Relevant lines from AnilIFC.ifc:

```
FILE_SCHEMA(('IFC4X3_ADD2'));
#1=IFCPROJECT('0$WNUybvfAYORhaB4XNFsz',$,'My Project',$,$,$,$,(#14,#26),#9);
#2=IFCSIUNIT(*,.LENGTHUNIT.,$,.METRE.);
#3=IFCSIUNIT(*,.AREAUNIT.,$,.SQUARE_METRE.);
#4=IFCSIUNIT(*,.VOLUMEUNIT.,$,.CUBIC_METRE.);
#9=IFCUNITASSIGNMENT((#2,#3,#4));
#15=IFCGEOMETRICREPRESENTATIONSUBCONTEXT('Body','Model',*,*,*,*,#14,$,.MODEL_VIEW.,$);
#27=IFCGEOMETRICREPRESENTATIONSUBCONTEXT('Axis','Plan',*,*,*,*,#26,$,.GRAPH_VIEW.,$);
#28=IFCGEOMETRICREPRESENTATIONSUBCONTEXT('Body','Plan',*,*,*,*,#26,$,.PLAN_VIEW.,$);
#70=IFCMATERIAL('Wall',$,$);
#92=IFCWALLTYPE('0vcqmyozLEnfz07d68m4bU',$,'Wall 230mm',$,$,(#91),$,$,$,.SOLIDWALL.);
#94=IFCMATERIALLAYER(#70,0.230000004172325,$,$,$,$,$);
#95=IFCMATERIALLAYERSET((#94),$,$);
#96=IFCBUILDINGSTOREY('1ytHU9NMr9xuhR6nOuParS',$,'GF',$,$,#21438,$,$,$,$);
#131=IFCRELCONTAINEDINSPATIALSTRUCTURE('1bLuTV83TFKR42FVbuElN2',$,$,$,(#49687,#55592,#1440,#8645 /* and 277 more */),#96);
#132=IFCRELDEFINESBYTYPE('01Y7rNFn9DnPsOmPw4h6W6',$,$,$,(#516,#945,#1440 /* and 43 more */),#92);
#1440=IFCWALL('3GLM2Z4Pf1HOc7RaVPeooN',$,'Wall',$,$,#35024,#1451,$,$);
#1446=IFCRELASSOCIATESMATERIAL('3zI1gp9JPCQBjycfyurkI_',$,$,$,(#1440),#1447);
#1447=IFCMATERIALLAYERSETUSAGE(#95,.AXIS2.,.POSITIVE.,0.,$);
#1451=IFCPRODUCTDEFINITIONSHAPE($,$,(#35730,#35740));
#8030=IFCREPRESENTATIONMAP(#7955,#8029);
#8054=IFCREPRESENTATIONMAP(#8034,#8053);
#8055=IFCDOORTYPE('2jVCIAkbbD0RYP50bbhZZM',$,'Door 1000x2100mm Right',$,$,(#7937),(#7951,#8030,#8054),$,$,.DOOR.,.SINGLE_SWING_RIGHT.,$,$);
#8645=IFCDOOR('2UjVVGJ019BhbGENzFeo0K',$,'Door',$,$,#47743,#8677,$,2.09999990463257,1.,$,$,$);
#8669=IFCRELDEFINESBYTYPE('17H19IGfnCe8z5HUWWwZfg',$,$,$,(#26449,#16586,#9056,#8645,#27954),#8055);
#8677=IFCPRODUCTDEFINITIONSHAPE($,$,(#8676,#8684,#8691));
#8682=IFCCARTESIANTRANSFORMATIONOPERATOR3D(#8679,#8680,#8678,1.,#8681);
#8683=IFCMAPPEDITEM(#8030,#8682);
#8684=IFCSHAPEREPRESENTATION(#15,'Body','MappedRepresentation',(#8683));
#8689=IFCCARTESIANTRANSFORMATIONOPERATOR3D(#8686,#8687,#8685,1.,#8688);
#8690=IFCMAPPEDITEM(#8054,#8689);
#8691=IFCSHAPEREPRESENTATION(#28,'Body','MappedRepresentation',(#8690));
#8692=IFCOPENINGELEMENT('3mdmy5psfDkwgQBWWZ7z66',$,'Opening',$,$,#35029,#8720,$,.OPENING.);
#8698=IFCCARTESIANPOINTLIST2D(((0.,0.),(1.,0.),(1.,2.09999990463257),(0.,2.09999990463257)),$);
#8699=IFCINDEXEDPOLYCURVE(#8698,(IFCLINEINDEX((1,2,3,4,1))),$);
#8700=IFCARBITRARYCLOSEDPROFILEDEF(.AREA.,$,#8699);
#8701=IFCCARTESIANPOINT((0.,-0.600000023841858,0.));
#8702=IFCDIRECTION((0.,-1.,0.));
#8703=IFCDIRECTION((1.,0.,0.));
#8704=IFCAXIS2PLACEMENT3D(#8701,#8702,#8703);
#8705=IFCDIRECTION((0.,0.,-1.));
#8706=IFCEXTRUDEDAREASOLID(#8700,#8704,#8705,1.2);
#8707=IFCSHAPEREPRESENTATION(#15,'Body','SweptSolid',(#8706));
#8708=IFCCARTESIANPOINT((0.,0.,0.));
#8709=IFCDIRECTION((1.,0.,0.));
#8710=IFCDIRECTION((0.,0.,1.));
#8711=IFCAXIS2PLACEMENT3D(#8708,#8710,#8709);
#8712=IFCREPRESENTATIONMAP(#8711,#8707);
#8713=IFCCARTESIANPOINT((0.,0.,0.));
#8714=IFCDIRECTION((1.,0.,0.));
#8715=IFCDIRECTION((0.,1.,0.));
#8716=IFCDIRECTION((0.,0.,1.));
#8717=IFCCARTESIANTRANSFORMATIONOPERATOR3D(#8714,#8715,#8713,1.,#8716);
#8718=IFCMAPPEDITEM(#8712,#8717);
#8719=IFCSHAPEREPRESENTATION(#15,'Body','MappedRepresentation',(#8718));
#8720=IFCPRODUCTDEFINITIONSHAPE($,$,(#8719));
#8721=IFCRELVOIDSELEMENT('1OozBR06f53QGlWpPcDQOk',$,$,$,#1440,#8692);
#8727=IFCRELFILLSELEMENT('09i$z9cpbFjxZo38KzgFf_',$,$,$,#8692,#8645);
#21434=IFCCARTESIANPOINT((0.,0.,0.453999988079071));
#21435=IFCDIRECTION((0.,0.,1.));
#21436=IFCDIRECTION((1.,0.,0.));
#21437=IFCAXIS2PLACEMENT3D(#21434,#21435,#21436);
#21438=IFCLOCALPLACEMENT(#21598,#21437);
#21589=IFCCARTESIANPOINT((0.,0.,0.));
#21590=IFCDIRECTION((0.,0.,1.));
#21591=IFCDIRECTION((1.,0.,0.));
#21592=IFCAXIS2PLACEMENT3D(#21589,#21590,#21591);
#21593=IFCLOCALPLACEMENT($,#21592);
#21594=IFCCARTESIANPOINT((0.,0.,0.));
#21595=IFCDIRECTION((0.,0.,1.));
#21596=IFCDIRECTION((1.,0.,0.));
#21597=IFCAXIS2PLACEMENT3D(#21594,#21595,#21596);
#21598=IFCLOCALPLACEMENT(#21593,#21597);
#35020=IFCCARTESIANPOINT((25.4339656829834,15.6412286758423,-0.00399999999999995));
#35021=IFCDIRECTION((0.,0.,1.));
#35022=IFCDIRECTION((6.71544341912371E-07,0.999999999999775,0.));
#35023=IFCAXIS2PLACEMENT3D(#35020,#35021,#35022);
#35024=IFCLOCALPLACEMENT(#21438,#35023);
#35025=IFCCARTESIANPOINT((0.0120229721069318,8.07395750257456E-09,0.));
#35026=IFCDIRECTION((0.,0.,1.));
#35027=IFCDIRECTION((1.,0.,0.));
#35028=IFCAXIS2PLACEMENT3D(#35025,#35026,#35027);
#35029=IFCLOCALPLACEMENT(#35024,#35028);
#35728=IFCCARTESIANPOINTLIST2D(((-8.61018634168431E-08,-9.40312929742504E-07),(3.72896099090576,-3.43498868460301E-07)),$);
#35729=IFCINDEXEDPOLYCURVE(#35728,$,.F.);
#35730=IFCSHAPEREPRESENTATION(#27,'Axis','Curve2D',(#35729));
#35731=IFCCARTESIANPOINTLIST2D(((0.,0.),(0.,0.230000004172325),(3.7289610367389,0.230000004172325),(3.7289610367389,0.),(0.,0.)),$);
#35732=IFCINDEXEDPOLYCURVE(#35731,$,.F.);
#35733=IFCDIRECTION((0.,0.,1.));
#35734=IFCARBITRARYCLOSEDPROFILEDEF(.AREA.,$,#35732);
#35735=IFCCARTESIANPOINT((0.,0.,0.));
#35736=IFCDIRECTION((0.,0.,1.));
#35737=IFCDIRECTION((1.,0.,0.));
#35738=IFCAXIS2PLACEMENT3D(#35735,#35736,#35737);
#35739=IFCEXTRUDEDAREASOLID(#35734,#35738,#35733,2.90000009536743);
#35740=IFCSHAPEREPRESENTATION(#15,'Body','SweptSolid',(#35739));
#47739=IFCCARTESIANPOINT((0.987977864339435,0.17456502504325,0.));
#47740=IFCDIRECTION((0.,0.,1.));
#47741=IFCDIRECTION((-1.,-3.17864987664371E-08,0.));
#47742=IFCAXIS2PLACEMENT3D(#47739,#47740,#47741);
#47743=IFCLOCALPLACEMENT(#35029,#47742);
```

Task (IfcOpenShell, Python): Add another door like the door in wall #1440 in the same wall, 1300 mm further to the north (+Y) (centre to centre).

```python
import ifcopenshell
import ifcopenshell.api.feature
import ifcopenshell.api.geometry
import ifcopenshell.api.root
import ifcopenshell.geom
import ifcopenshell.util.element
import ifcopenshell.util.placement
import ifcopenshell.util.shape
import ifcopenshell.util.unit

model = ifcopenshell.open("AnilIFC.ifc")
unit_scale = ifcopenshell.util.unit.calculate_unit_scale(model)
settings = ifcopenshell.geom.settings()


def volume(element):
    """Net volume in cubic metres, openings subtracted."""
    shape = ifcopenshell.geom.create_shape(settings, element)
    return ifcopenshell.util.shape.get_volume(shape.geometry)


door = model.by_guid("2UjVVGJ019BhbGENzFeo0K")
opening = door.FillsVoids[0].RelatingOpeningElement
wall = opening.VoidsElements[0].RelatingBuildingElement
before = volume(wall)
shift = ifcopenshell.util.placement.get_local_placement(wall.ObjectPlacement)[:3, 0] * 1.3 / unit_scale

# copy_class copies the void relationship, type, container and properties, but no geometry.
new_opening = ifcopenshell.api.root.copy_class(model, product=opening)
new_opening.Representation = ifcopenshell.util.element.copy_deep(
    model, opening.Representation, exclude=["IfcGeometricRepresentationContext", "IfcRepresentationMap"]
)
new_door = ifcopenshell.api.root.copy_class(model, product=door)
new_door.Representation = ifcopenshell.util.element.copy_deep(
    model, door.Representation, exclude=["IfcGeometricRepresentationContext", "IfcRepresentationMap"]
)
ifcopenshell.api.feature.add_filling(model, opening=new_opening, element=new_door)

for old, new in ((opening, new_opening), (door, new_door)):
    matrix = ifcopenshell.util.placement.get_local_placement(old.ObjectPlacement)
    matrix[:3, 3] += shift
    ifcopenshell.api.geometry.edit_object_placement(model, product=new, matrix=matrix, is_si=False)

after = volume(wall)

print(f"wall volume {before:.3f} -> {after:.3f} m3")

model.write("AnilIFC_updated.ifc")
```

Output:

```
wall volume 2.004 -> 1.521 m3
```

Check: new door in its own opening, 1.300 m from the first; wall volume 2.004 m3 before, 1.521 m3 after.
